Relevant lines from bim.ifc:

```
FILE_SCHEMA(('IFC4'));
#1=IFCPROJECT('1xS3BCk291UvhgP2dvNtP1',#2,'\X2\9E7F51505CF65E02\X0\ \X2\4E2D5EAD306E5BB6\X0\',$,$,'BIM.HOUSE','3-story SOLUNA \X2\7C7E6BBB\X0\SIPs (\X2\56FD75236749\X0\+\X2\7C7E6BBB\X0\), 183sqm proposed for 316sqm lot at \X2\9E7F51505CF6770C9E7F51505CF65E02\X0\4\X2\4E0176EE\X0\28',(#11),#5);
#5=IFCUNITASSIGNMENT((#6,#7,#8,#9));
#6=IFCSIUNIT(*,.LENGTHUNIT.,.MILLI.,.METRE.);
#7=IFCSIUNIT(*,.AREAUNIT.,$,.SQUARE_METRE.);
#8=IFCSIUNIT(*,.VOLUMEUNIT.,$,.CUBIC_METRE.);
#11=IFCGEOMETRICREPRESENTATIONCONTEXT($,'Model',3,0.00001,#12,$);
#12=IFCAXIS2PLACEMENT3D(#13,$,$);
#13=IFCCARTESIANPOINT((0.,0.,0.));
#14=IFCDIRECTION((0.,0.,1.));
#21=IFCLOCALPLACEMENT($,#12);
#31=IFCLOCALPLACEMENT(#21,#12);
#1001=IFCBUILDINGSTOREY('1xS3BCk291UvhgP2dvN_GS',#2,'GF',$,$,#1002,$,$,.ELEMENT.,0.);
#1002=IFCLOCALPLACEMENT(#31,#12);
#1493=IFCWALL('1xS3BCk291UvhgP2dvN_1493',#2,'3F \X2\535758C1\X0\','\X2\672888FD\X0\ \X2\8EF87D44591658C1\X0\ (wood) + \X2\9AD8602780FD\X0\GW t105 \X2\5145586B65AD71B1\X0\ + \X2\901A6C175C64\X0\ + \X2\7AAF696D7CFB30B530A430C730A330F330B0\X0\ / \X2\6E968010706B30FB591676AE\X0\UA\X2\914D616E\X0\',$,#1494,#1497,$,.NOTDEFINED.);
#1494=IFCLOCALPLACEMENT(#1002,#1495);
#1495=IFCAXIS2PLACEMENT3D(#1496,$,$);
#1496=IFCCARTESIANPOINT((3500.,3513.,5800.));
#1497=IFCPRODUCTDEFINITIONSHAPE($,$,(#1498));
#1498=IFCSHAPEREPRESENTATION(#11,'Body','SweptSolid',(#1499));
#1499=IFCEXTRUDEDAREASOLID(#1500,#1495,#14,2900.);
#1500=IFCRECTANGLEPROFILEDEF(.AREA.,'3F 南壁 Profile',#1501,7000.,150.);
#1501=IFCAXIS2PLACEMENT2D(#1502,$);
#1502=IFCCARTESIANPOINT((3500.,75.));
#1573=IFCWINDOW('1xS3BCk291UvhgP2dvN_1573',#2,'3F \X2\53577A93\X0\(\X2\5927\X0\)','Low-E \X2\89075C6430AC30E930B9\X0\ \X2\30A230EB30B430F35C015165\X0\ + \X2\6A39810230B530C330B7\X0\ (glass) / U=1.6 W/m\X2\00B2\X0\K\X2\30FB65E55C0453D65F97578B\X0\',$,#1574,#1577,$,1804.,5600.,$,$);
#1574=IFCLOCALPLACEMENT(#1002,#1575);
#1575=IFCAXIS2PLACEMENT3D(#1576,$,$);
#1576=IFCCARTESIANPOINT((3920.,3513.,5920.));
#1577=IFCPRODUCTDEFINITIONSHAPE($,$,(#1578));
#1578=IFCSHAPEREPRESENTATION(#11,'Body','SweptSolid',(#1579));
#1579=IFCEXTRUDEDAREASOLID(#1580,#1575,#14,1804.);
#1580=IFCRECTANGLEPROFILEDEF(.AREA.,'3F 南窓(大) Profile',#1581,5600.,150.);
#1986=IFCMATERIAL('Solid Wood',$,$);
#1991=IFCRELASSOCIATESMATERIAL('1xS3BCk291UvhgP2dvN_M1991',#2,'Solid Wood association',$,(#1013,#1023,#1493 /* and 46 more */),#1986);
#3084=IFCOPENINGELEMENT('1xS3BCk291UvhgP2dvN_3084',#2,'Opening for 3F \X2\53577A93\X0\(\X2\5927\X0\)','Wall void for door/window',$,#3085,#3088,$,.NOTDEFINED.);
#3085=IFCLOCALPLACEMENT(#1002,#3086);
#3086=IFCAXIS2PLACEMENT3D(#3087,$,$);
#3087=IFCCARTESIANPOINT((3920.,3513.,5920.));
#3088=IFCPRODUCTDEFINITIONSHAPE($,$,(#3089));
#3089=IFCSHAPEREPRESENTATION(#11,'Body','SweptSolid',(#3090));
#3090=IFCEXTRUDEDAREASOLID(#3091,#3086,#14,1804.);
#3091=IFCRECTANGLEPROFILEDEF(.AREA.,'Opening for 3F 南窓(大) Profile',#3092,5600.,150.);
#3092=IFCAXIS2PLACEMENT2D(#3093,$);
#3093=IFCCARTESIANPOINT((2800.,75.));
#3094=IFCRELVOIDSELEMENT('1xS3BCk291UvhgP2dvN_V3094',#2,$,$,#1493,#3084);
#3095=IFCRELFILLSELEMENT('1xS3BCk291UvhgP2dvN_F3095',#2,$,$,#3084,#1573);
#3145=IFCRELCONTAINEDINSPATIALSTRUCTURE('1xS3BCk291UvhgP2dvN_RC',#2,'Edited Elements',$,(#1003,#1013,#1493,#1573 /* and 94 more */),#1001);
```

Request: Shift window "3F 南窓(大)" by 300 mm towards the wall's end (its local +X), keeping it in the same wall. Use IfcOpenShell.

```python
import ifcopenshell
import ifcopenshell.api.geometry
import ifcopenshell.util.placement

model = ifcopenshell.open("bim.ifc")

window = model.by_guid("1xS3BCk291UvhgP2dvN_1573")
opening = window.FillsVoids[0].RelatingOpeningElement
wall = opening.VoidsElements[0].RelatingBuildingElement

wall_matrix = ifcopenshell.util.placement.get_local_placement(wall.ObjectPlacement)
shift = wall_matrix[:3, 0] * 300.0
before = ifcopenshell.util.placement.get_local_placement(window.ObjectPlacement)[:3, 3].copy()

# The window is not placed relative to its opening, so move both.
for product in (opening, window):
    matrix = ifcopenshell.util.placement.get_local_placement(product.ObjectPlacement)
    matrix[:3, 3] += shift
    ifcopenshell.api.geometry.edit_object_placement(model, product=product, matrix=matrix, is_si=False)

after = ifcopenshell.util.placement.get_local_placement(window.ObjectPlacement)[:3, 3]
print("window moved by", (after - before).round(3) + 0.0)

model.write("bim_updated.ifc")
```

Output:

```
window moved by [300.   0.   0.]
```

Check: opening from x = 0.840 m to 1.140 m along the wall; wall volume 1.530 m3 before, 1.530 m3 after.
